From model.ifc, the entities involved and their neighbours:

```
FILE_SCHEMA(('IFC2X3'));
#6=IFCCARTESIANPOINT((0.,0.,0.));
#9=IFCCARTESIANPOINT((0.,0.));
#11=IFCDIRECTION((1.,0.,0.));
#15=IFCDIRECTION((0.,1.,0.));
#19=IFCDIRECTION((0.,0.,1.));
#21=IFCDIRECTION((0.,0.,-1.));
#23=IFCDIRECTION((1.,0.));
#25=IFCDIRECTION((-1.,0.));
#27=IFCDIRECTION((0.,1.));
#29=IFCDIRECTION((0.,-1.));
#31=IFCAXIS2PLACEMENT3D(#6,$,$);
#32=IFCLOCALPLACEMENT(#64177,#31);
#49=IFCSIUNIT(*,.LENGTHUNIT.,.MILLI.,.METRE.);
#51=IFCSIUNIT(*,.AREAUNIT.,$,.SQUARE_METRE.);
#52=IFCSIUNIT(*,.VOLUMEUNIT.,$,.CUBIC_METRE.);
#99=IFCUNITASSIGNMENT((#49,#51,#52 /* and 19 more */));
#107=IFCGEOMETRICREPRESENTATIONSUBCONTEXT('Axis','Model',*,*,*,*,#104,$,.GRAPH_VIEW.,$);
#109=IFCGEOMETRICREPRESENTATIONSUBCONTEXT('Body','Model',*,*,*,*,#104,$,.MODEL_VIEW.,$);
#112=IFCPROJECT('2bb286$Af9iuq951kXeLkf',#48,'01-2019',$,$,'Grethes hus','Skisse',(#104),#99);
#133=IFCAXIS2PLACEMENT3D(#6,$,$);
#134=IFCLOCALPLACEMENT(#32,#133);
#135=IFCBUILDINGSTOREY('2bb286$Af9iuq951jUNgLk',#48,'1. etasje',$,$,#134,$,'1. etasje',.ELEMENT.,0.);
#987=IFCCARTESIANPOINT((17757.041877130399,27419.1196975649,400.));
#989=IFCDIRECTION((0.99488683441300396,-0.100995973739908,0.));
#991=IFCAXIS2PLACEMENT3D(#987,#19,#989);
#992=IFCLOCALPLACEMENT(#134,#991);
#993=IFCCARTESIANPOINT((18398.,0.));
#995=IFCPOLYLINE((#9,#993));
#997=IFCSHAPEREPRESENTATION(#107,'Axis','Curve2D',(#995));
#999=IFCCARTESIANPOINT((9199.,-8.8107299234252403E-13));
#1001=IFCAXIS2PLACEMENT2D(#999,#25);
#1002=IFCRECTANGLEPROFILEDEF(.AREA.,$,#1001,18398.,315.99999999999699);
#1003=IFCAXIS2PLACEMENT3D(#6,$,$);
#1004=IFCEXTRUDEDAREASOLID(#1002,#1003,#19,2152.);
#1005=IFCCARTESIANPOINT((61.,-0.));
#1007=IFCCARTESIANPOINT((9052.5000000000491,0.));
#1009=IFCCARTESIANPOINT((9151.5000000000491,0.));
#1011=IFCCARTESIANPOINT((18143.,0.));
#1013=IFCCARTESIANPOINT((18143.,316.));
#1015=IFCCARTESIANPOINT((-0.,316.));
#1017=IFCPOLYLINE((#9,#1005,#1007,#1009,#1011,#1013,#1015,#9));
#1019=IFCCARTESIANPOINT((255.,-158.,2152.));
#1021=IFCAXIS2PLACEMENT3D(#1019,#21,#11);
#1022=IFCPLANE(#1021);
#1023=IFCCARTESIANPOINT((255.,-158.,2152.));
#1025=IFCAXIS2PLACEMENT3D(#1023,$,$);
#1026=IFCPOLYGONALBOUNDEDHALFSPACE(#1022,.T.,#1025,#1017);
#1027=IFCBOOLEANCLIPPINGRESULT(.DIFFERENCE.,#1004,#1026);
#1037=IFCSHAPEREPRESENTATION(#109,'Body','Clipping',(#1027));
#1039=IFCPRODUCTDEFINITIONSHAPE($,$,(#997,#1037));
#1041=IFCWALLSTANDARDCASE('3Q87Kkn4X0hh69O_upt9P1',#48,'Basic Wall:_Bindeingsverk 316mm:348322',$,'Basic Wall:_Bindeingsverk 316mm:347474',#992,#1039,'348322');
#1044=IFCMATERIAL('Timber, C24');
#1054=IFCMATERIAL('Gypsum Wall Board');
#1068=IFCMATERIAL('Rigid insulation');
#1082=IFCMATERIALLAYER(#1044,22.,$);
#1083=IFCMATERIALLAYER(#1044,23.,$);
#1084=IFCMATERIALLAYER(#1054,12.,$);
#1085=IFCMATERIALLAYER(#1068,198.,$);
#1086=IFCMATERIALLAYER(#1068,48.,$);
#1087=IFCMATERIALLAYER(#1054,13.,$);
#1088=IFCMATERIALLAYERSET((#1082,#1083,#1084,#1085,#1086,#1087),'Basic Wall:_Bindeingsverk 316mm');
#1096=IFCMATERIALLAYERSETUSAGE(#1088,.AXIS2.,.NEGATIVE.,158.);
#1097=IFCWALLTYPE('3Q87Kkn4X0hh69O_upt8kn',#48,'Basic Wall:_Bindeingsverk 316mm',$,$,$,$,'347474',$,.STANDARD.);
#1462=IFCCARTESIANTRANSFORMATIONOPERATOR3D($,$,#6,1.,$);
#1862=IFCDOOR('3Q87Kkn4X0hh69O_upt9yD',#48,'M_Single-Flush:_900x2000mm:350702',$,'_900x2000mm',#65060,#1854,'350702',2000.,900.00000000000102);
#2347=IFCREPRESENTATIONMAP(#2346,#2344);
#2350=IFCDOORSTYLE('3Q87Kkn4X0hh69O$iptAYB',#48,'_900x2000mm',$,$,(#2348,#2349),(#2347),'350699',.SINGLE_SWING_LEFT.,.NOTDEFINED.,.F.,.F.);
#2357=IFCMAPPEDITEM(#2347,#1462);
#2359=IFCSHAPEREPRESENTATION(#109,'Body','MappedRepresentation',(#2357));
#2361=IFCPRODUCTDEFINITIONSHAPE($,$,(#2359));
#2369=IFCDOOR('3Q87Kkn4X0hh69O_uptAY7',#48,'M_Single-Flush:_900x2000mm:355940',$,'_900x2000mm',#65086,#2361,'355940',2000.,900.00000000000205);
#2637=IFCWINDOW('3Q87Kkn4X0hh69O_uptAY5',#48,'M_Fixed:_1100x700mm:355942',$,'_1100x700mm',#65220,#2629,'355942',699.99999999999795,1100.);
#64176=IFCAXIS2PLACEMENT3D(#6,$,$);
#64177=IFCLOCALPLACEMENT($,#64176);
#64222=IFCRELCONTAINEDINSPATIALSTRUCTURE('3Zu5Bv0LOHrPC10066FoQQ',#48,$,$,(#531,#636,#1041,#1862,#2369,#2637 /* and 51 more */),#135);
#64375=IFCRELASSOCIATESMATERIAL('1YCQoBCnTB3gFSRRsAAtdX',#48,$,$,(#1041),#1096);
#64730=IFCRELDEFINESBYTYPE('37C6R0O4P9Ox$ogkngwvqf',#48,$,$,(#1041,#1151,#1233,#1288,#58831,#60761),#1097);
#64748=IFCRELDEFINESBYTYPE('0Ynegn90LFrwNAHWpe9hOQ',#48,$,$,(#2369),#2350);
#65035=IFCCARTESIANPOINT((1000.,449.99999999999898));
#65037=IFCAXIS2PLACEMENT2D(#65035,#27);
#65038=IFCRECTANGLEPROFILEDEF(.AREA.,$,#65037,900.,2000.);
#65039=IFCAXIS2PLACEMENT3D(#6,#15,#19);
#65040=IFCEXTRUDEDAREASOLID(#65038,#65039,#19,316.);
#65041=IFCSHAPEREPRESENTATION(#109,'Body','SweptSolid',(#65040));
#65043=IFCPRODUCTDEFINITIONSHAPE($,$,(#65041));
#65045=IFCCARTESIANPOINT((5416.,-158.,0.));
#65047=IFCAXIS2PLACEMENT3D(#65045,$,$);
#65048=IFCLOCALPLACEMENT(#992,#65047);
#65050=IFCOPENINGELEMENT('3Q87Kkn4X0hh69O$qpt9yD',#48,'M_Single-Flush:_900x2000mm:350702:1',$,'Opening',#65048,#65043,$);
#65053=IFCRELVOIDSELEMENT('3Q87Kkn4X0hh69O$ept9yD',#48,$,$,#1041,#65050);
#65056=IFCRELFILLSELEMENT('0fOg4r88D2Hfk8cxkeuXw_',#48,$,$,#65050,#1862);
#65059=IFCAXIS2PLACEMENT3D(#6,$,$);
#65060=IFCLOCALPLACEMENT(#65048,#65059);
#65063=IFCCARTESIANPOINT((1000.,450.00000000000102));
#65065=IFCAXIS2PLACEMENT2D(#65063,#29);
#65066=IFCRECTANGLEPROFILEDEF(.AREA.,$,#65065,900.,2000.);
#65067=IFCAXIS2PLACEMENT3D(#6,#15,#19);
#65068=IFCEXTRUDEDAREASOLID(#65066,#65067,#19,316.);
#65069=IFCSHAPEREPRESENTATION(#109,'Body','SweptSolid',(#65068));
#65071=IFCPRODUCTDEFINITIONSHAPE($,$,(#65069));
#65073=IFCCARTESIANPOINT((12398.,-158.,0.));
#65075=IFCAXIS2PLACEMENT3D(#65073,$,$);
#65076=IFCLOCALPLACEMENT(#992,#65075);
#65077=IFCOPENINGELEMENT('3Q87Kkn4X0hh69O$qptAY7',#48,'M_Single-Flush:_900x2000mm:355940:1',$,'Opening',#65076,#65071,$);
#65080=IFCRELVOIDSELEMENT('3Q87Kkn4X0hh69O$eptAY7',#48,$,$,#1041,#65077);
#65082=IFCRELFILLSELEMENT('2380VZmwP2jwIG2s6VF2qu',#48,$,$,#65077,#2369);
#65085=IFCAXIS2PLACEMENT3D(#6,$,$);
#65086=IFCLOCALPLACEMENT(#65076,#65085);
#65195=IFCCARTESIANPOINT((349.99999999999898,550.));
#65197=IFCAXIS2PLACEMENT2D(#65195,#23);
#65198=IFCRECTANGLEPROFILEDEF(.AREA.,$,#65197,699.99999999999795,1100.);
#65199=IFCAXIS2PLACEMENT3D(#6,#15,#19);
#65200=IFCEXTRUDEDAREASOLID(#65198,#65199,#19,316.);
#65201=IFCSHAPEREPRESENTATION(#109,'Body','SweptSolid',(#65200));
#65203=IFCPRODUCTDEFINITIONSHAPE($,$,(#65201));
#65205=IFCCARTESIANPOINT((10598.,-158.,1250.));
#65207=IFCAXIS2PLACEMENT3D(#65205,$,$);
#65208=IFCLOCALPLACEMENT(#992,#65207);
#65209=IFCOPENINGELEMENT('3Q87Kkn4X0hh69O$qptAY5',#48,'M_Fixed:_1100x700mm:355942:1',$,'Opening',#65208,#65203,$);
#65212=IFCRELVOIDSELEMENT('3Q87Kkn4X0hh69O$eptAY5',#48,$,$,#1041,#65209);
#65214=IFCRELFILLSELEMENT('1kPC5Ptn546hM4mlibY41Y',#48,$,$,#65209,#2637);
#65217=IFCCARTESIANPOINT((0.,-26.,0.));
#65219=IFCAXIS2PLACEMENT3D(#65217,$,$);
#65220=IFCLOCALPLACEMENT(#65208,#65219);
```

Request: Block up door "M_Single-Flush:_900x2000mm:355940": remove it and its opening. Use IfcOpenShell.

```python
import ifcopenshell
import ifcopenshell.api.feature
import ifcopenshell.api.root
import ifcopenshell.geom
import ifcopenshell.util.shape

model = ifcopenshell.open("model.ifc")
settings = ifcopenshell.geom.settings()


def volume(element):
    """Net volume in cubic metres, openings subtracted."""
    shape = ifcopenshell.geom.create_shape(settings, element)
    return ifcopenshell.util.shape.get_volume(shape.geometry)


door = model.by_id(2369)
opening = door.FillsVoids[0].RelatingOpeningElement
wall = opening.VoidsElements[0].RelatingBuildingElement
before = volume(wall)

ifcopenshell.api.root.remove_product(model, product=door)
ifcopenshell.api.feature.remove_feature(model, feature=opening)

after = volume(wall)

print(f"wall volume {before:.3f} -> {after:.3f} m3")

model.write("model_edited.ifc")
```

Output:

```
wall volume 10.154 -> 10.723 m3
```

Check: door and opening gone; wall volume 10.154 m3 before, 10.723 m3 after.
